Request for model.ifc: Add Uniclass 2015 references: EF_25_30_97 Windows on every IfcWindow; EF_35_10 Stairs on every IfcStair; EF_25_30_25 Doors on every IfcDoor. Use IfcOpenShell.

First a look at what the model holds.

```python
import ifcopenshell

model = ifcopenshell.open("model.ifc")
print(model.schema)
print("classifications:", [c.Name for c in model.by_type("IfcClassification")])
for ifc_class in ("IfcDoor", "IfcRoof", "IfcStair", "IfcWall", "IfcWindow"):
    print(ifc_class, len(model.by_type(ifc_class)))
```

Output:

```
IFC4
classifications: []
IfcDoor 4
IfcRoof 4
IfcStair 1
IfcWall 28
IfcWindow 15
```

```python
import ifcopenshell
import ifcopenshell.api.classification

model = ifcopenshell.open("model.ifc")

system = ifcopenshell.api.classification.add_classification(model, classification="Uniclass 2015")

codes = {
    "IfcWindow": ("EF_25_30_97", "Windows"),
    "IfcStair": ("EF_35_10", "Stairs"),
    "IfcDoor": ("EF_25_30_25", "Doors"),
}
for ifc_class, (code, name) in codes.items():
    products = model.by_type(ifc_class)
    ifcopenshell.api.classification.add_reference(
        model, products=products, classification=system, identification=code, name=name
    )
    print(code, len(products))

model.write("model_rev.ifc")
```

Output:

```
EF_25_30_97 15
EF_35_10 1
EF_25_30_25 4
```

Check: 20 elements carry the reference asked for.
